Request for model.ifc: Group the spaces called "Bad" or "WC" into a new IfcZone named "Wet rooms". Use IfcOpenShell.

First a look at what the model holds.

```python
import ifcopenshell

model = ifcopenshell.open("model.ifc")
print(model.schema)
seen = {}
for space in model.by_type("IfcSpace"):
    seen[space.LongName] = seen.get(space.LongName, 0) + 1
for name, count in sorted(seen.items(), key=str):
    print(count, "x", name)
print("zones:", [z.Name for z in model.by_type("IfcZone")][:20])
```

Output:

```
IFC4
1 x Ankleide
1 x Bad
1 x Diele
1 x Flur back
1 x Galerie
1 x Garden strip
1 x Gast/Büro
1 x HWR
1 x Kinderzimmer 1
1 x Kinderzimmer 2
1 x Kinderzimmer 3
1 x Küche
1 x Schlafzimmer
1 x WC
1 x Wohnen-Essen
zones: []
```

```python
import ifcopenshell
import ifcopenshell.api.group
import ifcopenshell.api.root

model = ifcopenshell.open("model.ifc")

names = {"Bad", "WC"}
spaces = [s for s in model.by_type("IfcSpace") if s.LongName in names]

zone = ifcopenshell.api.root.create_entity(model, ifc_class="IfcZone", name="Wet rooms")
ifcopenshell.api.group.assign_group(model, products=spaces, group=zone)
print(len(spaces), "spaces in", zone.Name)

model.write("model_v2.ifc")
```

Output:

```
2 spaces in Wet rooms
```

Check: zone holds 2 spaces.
